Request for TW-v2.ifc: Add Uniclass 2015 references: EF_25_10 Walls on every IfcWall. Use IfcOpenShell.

First a look at what the model holds.

```python
import ifcopenshell

model = ifcopenshell.open("TW-v2.ifc")
print(model.schema)
print("classifications:", [c.Name for c in model.by_type("IfcClassification")])
for ifc_class in ("IfcDoor", "IfcRoof", "IfcStair", "IfcWall", "IfcWindow"):
    print(ifc_class, len(model.by_type(ifc_class)))
```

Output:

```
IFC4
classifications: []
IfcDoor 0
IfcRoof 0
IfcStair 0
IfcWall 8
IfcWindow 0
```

```python
import ifcopenshell
import ifcopenshell.api.classification

model = ifcopenshell.open("TW-v2.ifc")

system = ifcopenshell.api.classification.add_classification(model, classification="Uniclass 2015")

codes = {
    "IfcWall": ("EF_25_10", "Walls"),
}
for ifc_class, (code, name) in codes.items():
    products = model.by_type(ifc_class)
    ifcopenshell.api.classification.add_reference(
        model, products=products, classification=system, identification=code, name=name
    )
    print(code, len(products))

model.write("TW-v2-out.ifc")
```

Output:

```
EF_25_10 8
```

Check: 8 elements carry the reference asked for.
